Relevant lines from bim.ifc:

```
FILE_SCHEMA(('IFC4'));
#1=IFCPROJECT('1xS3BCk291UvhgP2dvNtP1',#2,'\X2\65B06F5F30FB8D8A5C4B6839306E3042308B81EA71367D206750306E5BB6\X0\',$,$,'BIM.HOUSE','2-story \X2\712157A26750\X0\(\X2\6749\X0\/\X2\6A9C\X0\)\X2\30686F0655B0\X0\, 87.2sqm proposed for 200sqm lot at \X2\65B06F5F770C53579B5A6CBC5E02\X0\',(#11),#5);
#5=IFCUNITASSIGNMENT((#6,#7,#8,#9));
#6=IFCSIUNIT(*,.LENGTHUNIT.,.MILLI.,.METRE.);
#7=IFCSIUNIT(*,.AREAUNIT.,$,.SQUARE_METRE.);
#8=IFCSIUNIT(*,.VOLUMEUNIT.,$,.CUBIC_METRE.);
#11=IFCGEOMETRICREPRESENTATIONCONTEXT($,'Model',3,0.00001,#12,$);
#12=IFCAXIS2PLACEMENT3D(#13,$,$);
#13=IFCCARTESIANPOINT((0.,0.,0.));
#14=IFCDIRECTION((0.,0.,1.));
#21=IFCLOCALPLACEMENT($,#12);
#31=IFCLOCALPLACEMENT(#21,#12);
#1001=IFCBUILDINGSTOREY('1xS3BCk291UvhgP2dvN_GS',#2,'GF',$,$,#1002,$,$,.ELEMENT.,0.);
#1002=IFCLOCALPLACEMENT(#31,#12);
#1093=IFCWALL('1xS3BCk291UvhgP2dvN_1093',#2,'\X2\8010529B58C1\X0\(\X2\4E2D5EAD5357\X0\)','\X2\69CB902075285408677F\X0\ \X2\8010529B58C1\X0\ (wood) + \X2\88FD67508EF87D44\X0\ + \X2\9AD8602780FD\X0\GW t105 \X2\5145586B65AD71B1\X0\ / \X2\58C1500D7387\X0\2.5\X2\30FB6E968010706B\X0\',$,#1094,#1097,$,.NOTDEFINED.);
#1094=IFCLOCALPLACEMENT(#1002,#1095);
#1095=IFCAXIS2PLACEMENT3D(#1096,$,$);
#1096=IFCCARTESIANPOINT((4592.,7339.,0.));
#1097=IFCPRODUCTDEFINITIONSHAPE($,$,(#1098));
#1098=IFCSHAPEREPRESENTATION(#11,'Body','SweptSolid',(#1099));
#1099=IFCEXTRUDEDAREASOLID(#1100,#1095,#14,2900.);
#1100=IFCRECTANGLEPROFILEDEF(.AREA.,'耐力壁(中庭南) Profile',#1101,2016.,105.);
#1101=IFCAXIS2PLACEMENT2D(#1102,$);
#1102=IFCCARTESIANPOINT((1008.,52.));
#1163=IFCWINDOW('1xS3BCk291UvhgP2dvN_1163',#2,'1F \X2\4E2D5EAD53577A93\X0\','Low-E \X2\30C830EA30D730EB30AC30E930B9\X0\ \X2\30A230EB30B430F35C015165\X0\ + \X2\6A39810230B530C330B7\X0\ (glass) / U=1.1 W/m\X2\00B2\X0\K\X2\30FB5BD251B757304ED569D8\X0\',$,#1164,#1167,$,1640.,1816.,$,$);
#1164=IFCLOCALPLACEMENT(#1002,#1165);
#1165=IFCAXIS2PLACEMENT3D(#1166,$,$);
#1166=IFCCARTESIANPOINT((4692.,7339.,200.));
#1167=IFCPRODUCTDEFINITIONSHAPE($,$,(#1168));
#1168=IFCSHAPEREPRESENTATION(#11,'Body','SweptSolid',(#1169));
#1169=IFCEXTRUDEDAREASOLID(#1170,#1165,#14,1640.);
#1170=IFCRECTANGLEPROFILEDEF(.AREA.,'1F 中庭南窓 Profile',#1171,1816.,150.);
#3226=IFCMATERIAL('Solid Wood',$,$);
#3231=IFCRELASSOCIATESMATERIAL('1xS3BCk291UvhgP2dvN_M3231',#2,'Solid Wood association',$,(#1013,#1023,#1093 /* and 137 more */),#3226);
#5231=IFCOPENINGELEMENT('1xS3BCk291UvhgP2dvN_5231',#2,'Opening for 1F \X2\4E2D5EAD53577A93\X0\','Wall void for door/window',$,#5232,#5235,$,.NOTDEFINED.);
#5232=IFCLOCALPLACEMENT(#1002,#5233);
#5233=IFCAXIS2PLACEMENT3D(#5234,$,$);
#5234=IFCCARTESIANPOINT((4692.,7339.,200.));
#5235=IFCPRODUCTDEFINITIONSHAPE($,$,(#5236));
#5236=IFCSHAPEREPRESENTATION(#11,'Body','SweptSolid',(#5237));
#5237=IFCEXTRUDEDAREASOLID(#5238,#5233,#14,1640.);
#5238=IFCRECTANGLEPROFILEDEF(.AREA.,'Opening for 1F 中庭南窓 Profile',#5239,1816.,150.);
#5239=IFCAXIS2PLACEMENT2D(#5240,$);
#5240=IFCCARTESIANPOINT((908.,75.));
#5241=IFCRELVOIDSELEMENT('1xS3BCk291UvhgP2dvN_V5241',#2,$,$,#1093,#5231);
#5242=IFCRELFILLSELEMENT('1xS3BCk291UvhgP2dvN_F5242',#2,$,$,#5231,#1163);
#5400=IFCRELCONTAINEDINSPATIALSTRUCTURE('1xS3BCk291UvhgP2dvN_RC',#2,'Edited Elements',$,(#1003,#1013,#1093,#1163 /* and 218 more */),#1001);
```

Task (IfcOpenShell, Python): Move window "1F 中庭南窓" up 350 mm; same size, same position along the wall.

```python
import numpy as np
import ifcopenshell
import ifcopenshell.api.geometry
import ifcopenshell.util.placement
import ifcopenshell.util.unit

model = ifcopenshell.open("bim.ifc")
unit_scale = ifcopenshell.util.unit.calculate_unit_scale(model)

window = model.by_id(1163)
opening = window.FillsVoids[0].RelatingOpeningElement
dz = 0.35 / unit_scale

shift = np.array([0.0, 0.0, dz])
# The window is not placed relative to its opening, so move both.
for product in (opening, window):
    matrix = ifcopenshell.util.placement.get_local_placement(product.ObjectPlacement)
    matrix[:3, 3] += shift
    ifcopenshell.api.geometry.edit_object_placement(model, product=product, matrix=matrix, is_si=False)

print(f"moved by {dz * unit_scale:+.3f} m")

model.write("bim_edited.ifc")
```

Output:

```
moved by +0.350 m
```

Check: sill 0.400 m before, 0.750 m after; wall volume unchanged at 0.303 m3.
